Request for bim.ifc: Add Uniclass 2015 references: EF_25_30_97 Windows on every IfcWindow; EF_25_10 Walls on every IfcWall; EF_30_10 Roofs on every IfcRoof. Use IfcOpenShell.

First a look at what the model holds.

```python
import ifcopenshell

model = ifcopenshell.open("bim.ifc")
print(model.schema)
print("classifications:", [c.Name for c in model.by_type("IfcClassification")])
for ifc_class in ("IfcDoor", "IfcRoof", "IfcStair", "IfcWall", "IfcWindow"):
    print(ifc_class, len(model.by_type(ifc_class)))
```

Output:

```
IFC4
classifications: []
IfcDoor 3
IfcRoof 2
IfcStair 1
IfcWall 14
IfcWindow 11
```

```python
import ifcopenshell
import ifcopenshell.api.classification

model = ifcopenshell.open("bim.ifc")

system = ifcopenshell.api.classification.add_classification(model, classification="Uniclass 2015")

codes = {
    "IfcWindow": ("EF_25_30_97", "Windows"),
    "IfcWall": ("EF_25_10", "Walls"),
    "IfcRoof": ("EF_30_10", "Roofs"),
}
for ifc_class, (code, name) in codes.items():
    products = model.by_type(ifc_class)
    ifcopenshell.api.classification.add_reference(
        model, products=products, classification=system, identification=code, name=name
    )
    print(code, len(products))

model.write("bim_v2.ifc")
```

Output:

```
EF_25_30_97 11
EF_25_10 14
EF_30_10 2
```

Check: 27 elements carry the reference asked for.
